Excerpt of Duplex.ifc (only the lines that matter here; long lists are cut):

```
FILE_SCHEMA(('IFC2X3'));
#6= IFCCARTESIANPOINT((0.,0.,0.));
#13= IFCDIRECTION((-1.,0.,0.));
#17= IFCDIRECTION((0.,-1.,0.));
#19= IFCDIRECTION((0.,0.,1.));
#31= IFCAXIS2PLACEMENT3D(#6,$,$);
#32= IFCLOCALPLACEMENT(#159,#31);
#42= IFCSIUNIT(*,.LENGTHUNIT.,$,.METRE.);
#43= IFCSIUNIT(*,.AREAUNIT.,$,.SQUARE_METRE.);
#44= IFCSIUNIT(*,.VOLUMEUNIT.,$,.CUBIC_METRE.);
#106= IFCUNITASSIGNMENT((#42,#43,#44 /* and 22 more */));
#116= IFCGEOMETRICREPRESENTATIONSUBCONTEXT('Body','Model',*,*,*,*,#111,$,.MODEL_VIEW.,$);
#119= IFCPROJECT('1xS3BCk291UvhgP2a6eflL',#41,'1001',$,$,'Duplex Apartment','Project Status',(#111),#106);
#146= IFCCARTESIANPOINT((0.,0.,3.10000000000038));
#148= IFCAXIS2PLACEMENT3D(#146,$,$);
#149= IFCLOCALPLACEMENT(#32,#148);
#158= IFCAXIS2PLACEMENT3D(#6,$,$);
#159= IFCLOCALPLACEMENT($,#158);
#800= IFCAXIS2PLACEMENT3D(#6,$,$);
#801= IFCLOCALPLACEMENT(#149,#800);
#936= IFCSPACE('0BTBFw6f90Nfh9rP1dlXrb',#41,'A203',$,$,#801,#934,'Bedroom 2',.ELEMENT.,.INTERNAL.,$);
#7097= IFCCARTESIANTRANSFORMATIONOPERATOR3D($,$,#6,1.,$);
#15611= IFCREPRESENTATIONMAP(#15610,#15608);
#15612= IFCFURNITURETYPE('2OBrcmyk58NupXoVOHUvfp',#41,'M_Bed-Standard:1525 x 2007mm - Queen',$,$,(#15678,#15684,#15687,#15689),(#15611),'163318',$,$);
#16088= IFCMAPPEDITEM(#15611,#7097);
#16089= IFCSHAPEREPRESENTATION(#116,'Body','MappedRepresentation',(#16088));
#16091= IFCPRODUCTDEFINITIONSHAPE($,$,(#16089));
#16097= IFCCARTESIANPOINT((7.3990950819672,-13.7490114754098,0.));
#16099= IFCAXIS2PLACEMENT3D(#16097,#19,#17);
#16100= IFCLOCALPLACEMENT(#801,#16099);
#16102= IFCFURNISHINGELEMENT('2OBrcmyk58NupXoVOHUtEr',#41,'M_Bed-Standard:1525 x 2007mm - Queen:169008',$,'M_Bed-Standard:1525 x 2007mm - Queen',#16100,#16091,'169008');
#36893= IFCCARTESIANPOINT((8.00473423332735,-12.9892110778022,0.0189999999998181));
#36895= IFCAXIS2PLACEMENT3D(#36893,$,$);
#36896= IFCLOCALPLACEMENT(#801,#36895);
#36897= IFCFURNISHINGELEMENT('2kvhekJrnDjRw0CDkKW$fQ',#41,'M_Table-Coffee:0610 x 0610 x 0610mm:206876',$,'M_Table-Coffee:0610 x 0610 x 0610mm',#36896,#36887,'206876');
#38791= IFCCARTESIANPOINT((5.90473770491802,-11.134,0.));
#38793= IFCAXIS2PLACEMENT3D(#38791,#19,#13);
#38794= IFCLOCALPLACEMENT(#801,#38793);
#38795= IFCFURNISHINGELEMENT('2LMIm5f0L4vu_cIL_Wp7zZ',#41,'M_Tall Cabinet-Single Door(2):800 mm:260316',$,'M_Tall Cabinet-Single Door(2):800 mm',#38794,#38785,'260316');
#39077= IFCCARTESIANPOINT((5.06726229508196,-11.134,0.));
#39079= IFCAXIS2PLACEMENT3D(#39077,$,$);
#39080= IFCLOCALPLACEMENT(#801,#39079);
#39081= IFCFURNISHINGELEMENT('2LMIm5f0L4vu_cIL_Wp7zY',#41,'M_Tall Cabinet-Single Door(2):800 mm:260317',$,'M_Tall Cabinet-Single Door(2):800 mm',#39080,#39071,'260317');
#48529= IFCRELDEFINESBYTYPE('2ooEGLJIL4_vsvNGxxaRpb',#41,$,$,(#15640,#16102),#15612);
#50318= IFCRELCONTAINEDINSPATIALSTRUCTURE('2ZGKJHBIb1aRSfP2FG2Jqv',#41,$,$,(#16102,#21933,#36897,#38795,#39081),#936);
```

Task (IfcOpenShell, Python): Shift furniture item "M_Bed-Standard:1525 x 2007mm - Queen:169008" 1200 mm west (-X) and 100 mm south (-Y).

```python
import ifcopenshell
import ifcopenshell.api.geometry
import ifcopenshell.util.placement
import ifcopenshell.util.unit

model = ifcopenshell.open("Duplex.ifc")
unit_scale = ifcopenshell.util.unit.calculate_unit_scale(model)

item = model.by_id(16102)
matrix = ifcopenshell.util.placement.get_local_placement(item.ObjectPlacement)
matrix[0, 3] -= 1.2 / unit_scale
matrix[1, 3] -= 0.1 / unit_scale
ifcopenshell.api.geometry.edit_object_placement(model, product=item, matrix=matrix, is_si=False)

print(ifcopenshell.util.placement.get_local_placement(item.ObjectPlacement).round(3) + 0.0)

model.write("Duplex_v2.ifc")
```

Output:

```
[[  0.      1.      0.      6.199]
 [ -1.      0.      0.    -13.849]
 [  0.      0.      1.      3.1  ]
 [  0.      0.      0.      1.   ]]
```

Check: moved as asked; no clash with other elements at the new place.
